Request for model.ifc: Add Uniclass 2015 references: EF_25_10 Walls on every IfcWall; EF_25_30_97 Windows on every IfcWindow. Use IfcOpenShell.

First a look at what the model holds.

```python
import ifcopenshell

model = ifcopenshell.open("model.ifc")
print(model.schema)
print("classifications:", [c.Name for c in model.by_type("IfcClassification")])
for ifc_class in ("IfcDoor", "IfcRoof", "IfcStair", "IfcWall", "IfcWindow"):
    print(ifc_class, len(model.by_type(ifc_class)))
```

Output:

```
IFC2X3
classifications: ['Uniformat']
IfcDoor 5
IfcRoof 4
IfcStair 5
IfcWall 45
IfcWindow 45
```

```python
import ifcopenshell
import ifcopenshell.api.classification

model = ifcopenshell.open("model.ifc")

# IFC2X3 requires Source and Edition and has no link from the project to the system.
system = model.create_entity("IfcClassification", Source="NBS", Edition="2015", Name="Uniclass 2015")

codes = {
    "IfcWall": ("EF_25_10", "Walls"),
    "IfcWindow": ("EF_25_30_97", "Windows"),
}
for ifc_class, (code, name) in codes.items():
    products = model.by_type(ifc_class)
    ifcopenshell.api.classification.add_reference(
        model, products=products, classification=system, identification=code, name=name
    )
    print(code, len(products))

model.write("model-out.ifc")
```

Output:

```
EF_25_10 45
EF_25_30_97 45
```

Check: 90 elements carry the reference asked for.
